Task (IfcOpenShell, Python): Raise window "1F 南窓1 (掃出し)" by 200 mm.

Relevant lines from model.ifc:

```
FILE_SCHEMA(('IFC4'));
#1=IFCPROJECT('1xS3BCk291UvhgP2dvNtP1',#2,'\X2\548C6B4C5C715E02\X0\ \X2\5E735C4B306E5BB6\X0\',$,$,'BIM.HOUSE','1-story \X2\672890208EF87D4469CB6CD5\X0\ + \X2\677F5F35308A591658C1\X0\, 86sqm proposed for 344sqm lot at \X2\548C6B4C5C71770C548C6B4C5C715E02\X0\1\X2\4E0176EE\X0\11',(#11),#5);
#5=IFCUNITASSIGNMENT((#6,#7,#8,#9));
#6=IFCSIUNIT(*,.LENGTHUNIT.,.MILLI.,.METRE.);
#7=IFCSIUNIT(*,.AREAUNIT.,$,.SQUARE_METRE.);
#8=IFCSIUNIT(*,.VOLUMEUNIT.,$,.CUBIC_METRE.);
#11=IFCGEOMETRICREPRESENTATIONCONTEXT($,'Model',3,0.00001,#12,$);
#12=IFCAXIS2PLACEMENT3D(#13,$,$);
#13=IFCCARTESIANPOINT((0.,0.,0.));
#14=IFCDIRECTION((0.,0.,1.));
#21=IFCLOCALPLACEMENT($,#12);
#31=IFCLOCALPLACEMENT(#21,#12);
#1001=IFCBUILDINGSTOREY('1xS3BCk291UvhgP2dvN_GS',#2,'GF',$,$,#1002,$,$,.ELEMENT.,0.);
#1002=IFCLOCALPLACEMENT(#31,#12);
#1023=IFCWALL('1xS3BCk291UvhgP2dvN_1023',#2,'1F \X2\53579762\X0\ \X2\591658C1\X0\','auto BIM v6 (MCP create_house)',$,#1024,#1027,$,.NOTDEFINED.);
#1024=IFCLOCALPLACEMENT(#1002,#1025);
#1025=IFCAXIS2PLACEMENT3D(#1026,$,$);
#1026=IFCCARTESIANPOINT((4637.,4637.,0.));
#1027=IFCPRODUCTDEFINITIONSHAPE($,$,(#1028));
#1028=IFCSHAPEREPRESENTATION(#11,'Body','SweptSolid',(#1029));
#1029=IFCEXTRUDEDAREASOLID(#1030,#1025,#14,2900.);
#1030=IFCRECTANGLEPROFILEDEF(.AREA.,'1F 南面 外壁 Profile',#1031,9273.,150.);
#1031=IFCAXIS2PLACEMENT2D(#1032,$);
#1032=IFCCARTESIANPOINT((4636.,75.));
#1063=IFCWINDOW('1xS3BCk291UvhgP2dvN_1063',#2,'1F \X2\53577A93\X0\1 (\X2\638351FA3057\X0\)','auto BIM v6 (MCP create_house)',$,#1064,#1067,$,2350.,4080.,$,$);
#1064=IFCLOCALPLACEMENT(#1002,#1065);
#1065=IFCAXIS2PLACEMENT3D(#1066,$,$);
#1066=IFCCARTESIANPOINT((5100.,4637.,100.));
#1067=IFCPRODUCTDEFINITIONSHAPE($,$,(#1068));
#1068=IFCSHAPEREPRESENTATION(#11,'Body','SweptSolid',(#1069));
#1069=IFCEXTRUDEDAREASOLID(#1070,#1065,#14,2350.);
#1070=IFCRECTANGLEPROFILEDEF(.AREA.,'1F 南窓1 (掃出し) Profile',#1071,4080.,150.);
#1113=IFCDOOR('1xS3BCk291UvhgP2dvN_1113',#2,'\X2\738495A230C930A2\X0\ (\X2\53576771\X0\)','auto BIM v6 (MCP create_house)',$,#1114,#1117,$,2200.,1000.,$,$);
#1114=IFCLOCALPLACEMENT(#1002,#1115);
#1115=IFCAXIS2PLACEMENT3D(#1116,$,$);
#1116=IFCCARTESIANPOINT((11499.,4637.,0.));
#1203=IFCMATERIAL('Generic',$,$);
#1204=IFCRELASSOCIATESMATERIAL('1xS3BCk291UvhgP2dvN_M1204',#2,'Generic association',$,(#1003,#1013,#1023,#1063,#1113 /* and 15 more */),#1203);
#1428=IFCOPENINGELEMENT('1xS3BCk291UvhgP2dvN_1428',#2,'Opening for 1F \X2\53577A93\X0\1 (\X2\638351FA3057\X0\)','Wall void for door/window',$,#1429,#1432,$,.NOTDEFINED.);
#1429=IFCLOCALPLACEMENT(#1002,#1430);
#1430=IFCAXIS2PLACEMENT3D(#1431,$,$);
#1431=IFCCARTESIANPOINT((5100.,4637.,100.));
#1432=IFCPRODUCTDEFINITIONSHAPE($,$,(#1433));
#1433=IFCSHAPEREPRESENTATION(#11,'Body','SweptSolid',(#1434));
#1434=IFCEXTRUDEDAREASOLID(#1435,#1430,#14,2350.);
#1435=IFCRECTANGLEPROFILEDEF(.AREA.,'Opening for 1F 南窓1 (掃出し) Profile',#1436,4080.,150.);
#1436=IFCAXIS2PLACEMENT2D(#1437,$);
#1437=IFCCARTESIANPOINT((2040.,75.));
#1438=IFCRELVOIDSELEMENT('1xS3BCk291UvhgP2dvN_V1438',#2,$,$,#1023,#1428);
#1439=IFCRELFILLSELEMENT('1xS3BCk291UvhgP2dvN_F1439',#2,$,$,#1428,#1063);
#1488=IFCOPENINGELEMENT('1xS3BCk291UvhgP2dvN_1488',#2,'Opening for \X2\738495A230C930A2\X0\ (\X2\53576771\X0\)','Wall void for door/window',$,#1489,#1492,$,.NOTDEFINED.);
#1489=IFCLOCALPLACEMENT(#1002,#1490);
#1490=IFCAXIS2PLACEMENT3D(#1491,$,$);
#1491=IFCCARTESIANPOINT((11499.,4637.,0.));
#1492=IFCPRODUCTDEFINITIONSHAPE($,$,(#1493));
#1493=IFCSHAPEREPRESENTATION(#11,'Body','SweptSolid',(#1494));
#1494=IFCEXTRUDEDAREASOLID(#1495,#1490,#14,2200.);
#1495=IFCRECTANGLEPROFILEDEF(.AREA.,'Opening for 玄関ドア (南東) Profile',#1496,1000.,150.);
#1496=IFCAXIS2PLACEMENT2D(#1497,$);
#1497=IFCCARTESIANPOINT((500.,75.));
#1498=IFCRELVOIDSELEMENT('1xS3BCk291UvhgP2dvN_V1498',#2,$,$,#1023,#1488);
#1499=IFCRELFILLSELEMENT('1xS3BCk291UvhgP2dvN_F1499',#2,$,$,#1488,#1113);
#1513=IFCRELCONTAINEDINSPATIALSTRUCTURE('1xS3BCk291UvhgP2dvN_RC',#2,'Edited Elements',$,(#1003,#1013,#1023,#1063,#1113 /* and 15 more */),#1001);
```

```python
import numpy as np
import ifcopenshell
import ifcopenshell.api.geometry
import ifcopenshell.util.placement
import ifcopenshell.util.unit

model = ifcopenshell.open("model.ifc")
unit_scale = ifcopenshell.util.unit.calculate_unit_scale(model)

window = model.by_guid("1xS3BCk291UvhgP2dvN_1063")
opening = window.FillsVoids[0].RelatingOpeningElement
dz = 0.2 / unit_scale

shift = np.array([0.0, 0.0, dz])
# The window is not placed relative to its opening, so move both.
for product in (opening, window):
    matrix = ifcopenshell.util.placement.get_local_placement(product.ObjectPlacement)
    matrix[:3, 3] += shift
    ifcopenshell.api.geometry.edit_object_placement(model, product=product, matrix=matrix, is_si=False)

print(f"moved by {dz * unit_scale:+.3f} m")

model.write("model_updated.ifc")
```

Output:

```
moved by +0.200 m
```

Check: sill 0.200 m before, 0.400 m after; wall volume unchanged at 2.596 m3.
